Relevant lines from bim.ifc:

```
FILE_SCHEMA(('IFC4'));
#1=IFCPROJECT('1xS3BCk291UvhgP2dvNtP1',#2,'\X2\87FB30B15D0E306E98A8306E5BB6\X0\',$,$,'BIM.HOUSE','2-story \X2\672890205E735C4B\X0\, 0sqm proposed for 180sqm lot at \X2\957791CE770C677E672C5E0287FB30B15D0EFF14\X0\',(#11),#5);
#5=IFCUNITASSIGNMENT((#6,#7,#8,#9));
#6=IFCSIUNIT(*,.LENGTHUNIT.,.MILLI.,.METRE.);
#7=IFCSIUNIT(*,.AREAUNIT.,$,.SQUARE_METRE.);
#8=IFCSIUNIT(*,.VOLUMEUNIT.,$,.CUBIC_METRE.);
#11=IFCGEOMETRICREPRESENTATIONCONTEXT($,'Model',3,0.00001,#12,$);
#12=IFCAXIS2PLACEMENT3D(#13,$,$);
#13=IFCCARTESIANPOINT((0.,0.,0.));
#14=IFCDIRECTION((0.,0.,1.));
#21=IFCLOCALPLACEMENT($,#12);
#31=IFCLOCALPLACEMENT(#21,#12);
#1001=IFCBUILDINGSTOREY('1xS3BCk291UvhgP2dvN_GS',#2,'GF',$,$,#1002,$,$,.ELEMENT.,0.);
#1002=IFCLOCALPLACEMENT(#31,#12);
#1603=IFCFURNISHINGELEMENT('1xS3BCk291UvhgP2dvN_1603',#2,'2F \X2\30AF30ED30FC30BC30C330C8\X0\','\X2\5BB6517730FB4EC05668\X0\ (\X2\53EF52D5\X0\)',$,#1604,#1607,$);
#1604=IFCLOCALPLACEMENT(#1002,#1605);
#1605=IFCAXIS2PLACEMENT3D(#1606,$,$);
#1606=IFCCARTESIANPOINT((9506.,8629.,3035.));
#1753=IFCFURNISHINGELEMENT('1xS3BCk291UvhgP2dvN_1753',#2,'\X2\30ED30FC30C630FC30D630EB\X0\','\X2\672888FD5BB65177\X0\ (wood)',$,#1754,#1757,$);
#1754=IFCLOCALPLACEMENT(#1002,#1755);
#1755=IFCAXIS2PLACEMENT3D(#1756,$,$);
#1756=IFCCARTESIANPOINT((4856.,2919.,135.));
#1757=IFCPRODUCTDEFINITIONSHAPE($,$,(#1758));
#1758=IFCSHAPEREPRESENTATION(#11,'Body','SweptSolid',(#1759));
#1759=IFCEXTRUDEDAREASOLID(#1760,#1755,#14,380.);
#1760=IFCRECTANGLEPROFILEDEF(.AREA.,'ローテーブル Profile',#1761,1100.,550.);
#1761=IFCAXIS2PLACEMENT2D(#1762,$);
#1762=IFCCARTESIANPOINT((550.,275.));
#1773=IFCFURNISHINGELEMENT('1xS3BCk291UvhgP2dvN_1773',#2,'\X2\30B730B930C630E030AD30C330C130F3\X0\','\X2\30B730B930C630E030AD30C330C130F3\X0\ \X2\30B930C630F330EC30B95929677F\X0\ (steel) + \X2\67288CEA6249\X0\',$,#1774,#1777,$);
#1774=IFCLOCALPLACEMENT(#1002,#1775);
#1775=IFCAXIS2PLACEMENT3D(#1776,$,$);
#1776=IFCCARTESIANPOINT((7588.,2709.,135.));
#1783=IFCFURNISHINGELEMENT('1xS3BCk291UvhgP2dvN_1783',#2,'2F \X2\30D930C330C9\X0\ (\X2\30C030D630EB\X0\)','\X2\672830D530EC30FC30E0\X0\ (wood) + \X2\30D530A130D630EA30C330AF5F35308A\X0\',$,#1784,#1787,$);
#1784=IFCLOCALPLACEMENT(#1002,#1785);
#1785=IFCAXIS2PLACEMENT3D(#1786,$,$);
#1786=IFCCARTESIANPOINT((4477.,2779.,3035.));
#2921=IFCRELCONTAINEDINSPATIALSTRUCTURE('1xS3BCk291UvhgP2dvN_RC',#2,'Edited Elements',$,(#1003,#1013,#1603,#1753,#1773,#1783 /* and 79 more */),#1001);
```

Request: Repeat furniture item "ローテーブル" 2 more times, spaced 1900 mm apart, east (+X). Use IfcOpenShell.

```python
import numpy as np
import ifcopenshell
import ifcopenshell.api.geometry
import ifcopenshell.api.root
import ifcopenshell.util.element
import ifcopenshell.util.placement
import ifcopenshell.util.unit

model = ifcopenshell.open("bim.ifc")
unit_scale = ifcopenshell.util.unit.calculate_unit_scale(model)


def reuse_history(source, copy):
    """copy_class also copies each property set's owner history, people and application; keep the originals."""
    for rel in copy.IsDefinedBy:
        if rel.is_a("IfcRelDefinesByProperties") and (history := rel.RelatingPropertyDefinition.OwnerHistory):
            rel.RelatingPropertyDefinition.OwnerHistory = source.OwnerHistory
            ifcopenshell.util.element.remove_deep2(model, history)


source = model.by_id(1753)
base = ifcopenshell.util.placement.get_local_placement(source.ObjectPlacement)
step = np.array([1.0, 0.0, 0.0]) * 1.9 / unit_scale

for i in range(1, 3):
    copy = ifcopenshell.api.root.copy_class(model, product=source)
    copy.Representation = ifcopenshell.util.element.copy_deep(
        model, source.Representation, exclude=["IfcGeometricRepresentationContext", "IfcRepresentationMap"]
    )
    reuse_history(source, copy)
    matrix = base.copy()
    matrix[:3, 3] += i * step
    print("added at", matrix[:3, 3].round(3) + 0.0)
    ifcopenshell.api.geometry.edit_object_placement(model, product=copy, matrix=matrix, is_si=False)

model.write("bim_v2.ifc")
```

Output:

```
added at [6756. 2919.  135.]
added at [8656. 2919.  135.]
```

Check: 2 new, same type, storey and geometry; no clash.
